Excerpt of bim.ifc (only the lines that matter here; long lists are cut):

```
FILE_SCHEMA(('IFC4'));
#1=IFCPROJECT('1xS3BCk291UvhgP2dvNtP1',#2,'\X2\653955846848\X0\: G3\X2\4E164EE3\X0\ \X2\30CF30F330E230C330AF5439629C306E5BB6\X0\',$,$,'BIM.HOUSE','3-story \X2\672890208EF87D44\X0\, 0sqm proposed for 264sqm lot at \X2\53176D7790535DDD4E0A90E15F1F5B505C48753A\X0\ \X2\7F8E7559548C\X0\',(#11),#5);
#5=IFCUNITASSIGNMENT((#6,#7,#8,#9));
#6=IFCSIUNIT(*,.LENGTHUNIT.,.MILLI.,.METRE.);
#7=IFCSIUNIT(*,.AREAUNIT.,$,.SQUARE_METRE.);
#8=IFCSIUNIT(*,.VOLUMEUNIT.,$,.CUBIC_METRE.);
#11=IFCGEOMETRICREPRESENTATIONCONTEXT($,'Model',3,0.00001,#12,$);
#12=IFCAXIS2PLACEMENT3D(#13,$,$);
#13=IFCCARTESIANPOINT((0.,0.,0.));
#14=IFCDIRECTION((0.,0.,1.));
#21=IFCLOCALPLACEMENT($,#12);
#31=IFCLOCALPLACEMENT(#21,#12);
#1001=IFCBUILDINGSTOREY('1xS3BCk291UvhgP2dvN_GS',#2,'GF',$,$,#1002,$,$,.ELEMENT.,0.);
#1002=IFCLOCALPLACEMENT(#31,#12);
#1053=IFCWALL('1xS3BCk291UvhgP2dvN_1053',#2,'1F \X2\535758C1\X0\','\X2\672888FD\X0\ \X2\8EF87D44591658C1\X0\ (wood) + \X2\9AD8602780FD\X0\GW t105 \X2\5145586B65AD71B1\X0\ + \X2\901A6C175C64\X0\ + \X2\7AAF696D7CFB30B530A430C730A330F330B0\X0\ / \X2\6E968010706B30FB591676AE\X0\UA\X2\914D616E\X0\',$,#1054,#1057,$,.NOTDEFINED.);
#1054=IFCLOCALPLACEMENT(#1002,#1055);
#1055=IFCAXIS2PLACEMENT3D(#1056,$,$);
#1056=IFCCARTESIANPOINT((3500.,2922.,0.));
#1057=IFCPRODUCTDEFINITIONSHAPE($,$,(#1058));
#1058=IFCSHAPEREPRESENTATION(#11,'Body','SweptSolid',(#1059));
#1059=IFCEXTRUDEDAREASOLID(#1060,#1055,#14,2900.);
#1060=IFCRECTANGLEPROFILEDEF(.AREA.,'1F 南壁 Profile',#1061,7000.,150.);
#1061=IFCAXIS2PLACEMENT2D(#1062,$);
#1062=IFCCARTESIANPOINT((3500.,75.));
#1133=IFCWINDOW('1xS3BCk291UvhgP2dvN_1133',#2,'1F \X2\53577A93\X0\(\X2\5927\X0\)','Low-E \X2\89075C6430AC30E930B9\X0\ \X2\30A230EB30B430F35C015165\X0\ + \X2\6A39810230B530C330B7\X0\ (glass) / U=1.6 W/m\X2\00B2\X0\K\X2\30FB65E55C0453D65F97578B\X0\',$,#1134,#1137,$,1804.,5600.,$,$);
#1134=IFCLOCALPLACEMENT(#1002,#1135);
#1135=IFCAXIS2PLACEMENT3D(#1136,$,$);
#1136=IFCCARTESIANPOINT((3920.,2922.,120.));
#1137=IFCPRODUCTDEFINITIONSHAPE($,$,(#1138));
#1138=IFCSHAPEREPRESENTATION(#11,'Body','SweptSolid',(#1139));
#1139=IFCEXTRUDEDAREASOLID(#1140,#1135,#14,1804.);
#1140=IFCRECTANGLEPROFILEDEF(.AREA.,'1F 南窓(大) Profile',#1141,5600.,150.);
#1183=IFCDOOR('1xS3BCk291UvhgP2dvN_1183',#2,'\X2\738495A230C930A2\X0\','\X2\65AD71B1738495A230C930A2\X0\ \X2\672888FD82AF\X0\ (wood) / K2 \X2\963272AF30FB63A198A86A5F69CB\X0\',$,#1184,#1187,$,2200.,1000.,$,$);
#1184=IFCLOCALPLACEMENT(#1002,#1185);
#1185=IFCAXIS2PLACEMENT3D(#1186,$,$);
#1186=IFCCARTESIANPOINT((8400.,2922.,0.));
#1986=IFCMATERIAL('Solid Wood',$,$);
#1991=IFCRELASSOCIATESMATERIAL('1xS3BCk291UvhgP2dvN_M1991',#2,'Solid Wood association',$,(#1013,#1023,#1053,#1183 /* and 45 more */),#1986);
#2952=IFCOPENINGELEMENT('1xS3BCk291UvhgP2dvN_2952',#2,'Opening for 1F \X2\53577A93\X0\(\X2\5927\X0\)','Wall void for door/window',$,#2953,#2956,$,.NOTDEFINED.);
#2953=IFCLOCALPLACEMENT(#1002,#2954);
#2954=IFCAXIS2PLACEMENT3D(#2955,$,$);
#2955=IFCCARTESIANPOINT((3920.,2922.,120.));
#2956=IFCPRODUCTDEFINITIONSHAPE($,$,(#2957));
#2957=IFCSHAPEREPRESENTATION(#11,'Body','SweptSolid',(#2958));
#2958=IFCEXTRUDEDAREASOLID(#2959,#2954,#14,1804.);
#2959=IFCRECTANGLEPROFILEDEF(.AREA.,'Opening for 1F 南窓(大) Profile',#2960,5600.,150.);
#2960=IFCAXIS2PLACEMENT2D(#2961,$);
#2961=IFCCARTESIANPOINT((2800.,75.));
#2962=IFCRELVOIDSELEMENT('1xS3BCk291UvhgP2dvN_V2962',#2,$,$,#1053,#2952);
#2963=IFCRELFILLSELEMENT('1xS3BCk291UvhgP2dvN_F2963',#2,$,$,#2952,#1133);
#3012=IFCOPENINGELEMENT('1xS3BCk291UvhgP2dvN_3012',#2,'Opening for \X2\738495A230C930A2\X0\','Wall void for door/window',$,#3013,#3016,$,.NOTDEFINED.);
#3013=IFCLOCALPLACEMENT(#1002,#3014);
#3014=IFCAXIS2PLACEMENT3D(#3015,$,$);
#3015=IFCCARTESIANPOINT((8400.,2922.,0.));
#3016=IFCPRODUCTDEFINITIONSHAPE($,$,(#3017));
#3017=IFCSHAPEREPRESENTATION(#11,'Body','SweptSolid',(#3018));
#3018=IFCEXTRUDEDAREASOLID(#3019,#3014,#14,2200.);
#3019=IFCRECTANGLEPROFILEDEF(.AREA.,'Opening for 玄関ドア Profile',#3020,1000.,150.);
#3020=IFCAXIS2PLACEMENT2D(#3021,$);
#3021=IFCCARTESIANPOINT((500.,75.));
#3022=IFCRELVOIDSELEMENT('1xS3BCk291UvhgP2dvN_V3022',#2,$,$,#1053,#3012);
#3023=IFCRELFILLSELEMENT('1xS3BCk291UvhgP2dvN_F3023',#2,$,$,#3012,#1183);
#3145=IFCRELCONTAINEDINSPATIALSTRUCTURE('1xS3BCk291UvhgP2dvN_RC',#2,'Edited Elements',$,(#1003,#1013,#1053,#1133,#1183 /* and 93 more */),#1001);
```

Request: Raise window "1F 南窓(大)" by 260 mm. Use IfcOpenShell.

```python
import numpy as np
import ifcopenshell
import ifcopenshell.api.geometry
import ifcopenshell.util.placement
import ifcopenshell.util.unit

model = ifcopenshell.open("bim.ifc")
unit_scale = ifcopenshell.util.unit.calculate_unit_scale(model)

window = model.by_guid("1xS3BCk291UvhgP2dvN_1133")
opening = window.FillsVoids[0].RelatingOpeningElement
dz = 260.0

shift = np.array([0.0, 0.0, dz])
# The window is not placed relative to its opening, so move both.
for product in (opening, window):
    matrix = ifcopenshell.util.placement.get_local_placement(product.ObjectPlacement)
    matrix[:3, 3] += shift
    ifcopenshell.api.geometry.edit_object_placement(model, product=product, matrix=matrix, is_si=False)

print(f"moved by {dz * unit_scale:+.3f} m")

model.write("bim_v2.ifc")
```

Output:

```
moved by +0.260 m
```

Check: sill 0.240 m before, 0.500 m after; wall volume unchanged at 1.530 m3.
